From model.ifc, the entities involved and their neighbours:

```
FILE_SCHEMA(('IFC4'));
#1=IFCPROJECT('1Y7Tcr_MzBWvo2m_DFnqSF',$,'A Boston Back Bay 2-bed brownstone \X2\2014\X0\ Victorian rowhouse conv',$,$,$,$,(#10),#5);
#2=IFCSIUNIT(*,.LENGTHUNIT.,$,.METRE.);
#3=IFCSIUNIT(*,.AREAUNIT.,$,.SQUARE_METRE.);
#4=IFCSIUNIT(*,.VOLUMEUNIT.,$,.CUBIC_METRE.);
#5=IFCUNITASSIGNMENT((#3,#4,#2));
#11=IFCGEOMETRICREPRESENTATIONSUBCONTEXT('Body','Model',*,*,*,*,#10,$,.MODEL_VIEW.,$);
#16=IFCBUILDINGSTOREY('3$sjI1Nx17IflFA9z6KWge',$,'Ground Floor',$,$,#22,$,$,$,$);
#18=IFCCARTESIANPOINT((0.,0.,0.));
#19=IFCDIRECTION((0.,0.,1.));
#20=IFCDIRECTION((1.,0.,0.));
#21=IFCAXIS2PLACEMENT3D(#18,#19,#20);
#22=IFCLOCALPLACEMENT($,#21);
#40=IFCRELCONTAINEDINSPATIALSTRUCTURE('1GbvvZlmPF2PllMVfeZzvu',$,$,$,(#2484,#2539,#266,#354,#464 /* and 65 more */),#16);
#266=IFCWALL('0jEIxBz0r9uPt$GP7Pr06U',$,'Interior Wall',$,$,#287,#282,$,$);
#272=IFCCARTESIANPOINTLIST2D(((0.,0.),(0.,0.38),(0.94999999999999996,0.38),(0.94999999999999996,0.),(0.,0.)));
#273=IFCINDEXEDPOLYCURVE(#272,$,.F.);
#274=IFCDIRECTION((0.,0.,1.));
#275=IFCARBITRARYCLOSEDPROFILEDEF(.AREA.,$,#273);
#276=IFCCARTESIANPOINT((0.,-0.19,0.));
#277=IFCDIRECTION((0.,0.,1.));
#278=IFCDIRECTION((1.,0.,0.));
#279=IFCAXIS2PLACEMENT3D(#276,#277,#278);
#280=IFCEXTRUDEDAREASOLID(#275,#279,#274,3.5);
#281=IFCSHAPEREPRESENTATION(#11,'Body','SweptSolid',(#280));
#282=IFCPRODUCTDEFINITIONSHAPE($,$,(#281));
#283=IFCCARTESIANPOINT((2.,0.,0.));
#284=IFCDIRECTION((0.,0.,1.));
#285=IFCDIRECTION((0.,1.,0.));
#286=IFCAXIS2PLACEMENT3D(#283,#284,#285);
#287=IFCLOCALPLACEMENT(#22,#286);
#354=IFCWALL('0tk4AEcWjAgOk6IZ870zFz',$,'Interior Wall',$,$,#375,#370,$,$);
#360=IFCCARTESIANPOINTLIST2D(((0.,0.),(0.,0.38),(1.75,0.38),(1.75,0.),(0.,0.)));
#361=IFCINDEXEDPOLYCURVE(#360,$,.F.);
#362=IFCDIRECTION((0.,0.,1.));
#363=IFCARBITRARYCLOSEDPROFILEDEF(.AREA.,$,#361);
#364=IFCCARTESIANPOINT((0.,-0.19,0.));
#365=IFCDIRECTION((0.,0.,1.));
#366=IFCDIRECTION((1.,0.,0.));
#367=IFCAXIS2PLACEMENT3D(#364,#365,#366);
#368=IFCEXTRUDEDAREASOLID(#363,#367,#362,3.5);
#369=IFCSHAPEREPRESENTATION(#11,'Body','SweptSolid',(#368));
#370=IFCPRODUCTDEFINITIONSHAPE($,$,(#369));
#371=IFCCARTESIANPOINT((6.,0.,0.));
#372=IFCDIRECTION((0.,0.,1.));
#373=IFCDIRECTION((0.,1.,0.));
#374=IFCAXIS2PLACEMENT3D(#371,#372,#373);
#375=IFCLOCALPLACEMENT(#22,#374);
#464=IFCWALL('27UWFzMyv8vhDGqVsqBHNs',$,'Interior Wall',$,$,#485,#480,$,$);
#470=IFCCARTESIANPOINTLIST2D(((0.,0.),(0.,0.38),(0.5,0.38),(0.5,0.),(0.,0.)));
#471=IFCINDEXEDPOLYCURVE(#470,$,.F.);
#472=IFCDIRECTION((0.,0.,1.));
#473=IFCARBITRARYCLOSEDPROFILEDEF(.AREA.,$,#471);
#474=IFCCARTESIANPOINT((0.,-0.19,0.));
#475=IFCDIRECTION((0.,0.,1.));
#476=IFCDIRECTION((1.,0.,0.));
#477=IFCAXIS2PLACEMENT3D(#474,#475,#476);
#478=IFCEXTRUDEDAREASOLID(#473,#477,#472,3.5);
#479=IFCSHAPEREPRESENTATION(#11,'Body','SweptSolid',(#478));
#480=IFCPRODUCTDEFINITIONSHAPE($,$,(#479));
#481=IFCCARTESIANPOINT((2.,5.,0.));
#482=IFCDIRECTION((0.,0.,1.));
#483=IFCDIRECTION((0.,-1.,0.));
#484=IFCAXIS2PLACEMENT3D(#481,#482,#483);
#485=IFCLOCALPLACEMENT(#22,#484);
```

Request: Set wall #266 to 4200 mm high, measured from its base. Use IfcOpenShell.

```python
import ifcopenshell
import ifcopenshell.geom
import ifcopenshell.util.representation
import ifcopenshell.util.shape

model = ifcopenshell.open("model.ifc")
settings = ifcopenshell.geom.settings()


def volume(element):
    """Net volume in cubic metres, openings subtracted."""
    shape = ifcopenshell.geom.create_shape(settings, element)
    return ifcopenshell.util.shape.get_volume(shape.geometry)


wall = model.by_id(266)
before = volume(wall)

body = ifcopenshell.util.representation.get_representation(wall, "Model", "Body")
solid = body.Items[0]
old_height = solid.Depth
solid.Depth = 4.2
after = volume(wall)

print(f"height {old_height:g} -> {solid.Depth:g}, volume {before:.3f} -> {after:.3f} m3")

model.write("model_rev.ifc")
```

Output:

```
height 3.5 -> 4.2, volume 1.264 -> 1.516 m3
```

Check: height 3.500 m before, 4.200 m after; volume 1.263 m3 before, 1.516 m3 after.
